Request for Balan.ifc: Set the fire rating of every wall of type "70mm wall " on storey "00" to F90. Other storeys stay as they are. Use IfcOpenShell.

First a look at what the model holds.

```python
import ifcopenshell
import ifcopenshell.util.element

model = ifcopenshell.open("Balan.ifc")
print(model.schema)
storey = next(s for s in model.by_type("IfcBuildingStorey") if s.Name == "00")
walls = [e for e in ifcopenshell.util.element.get_decomposition(storey) if e.is_a("IfcWall")]
seen = {}
for e in walls:
    element_type = ifcopenshell.util.element.get_type(e)
    key = (element_type.Name if element_type != e and element_type else None, ifcopenshell.util.element.get_pset(e, "Pset_WallCommon", "FireRating"))
    seen[key] = seen.get(key, 0) + 1
for (name, value), count in sorted(seen.items(), key=str):
    print(count, "x", name, "|", value)
```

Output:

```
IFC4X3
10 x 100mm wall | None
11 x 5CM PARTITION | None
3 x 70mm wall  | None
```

```python
import ifcopenshell
import ifcopenshell.api.pset
import ifcopenshell.util.element

model = ifcopenshell.open("Balan.ifc")

storey = next(s for s in model.by_type("IfcBuildingStorey") if s.Name == "00")
walls = [e for e in ifcopenshell.util.element.get_decomposition(storey) if e.is_a("IfcWall")]

count = 0
for e in walls:
    element_type = ifcopenshell.util.element.get_type(e)
    if element_type in (None, e) or element_type.Name != "70mm wall ":
        continue
    # add_pset returns the element's existing set when there is one.
    pset = ifcopenshell.api.pset.add_pset(model, product=e, name="Pset_WallCommon")
    ifcopenshell.api.pset.edit_pset(model, pset=pset, properties={"FireRating": "F90"})
    count += 1

print(count, "walls updated")

model.write("Balan_rev.ifc")
```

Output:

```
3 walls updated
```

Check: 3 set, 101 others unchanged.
